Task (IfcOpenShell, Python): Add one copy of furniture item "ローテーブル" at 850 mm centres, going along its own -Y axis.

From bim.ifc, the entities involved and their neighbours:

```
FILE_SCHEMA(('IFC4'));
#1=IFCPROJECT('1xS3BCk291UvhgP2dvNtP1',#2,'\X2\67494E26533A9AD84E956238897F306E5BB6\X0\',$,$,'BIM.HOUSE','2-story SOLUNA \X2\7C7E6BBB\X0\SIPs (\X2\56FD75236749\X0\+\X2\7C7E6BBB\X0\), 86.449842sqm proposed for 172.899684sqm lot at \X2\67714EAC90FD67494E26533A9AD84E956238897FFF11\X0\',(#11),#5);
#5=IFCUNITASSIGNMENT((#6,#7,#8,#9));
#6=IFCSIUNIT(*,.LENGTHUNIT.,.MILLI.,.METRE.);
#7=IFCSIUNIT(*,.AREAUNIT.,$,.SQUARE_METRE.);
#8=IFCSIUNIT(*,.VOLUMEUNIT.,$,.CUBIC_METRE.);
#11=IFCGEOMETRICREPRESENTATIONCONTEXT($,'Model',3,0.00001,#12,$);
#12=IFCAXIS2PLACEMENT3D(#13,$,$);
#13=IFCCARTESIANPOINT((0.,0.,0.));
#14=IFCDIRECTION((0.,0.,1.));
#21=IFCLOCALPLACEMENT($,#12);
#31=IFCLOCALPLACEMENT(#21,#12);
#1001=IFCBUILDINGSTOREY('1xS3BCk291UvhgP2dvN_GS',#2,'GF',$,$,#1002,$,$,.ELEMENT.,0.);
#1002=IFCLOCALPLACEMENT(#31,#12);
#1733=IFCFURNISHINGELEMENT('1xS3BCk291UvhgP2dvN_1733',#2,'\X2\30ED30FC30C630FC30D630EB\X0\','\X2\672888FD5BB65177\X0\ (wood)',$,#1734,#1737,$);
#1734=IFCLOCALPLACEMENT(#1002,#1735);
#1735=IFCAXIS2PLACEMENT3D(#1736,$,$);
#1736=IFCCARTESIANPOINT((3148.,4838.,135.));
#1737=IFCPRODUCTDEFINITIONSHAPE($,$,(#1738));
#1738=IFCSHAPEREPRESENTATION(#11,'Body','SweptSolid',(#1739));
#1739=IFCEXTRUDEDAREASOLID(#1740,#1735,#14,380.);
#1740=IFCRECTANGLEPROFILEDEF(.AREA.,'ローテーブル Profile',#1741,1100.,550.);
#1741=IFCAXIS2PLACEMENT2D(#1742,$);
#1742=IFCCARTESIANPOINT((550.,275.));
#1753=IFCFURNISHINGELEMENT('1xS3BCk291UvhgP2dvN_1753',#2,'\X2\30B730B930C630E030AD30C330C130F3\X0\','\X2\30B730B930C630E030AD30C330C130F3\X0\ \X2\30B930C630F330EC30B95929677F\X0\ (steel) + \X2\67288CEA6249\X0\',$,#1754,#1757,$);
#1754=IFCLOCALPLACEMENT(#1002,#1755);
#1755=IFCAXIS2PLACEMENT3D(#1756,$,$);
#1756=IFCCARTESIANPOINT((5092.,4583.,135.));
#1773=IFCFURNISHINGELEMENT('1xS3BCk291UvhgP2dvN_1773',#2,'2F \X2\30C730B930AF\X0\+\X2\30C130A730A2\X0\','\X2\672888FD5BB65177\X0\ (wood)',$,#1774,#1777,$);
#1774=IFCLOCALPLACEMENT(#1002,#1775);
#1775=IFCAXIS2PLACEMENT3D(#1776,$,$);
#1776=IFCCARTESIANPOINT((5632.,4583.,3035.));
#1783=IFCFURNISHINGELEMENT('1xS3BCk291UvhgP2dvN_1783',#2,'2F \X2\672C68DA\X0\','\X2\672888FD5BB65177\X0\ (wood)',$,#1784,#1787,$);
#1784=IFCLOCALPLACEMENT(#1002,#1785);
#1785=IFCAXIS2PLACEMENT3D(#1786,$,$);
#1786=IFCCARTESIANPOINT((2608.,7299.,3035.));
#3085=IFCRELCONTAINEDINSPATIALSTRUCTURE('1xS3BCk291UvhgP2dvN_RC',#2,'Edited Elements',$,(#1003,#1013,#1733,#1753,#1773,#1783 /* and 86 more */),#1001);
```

```python
import ifcopenshell
import ifcopenshell.api.geometry
import ifcopenshell.api.root
import ifcopenshell.util.element
import ifcopenshell.util.placement
import ifcopenshell.util.unit

model = ifcopenshell.open("bim.ifc")
unit_scale = ifcopenshell.util.unit.calculate_unit_scale(model)


def reuse_history(source, copy):
    """copy_class also copies each property set's owner history, people and application; keep the originals."""
    for rel in copy.IsDefinedBy:
        if rel.is_a("IfcRelDefinesByProperties") and (history := rel.RelatingPropertyDefinition.OwnerHistory):
            rel.RelatingPropertyDefinition.OwnerHistory = source.OwnerHistory
            ifcopenshell.util.element.remove_deep2(model, history)


source = model.by_id(1733)
base = ifcopenshell.util.placement.get_local_placement(source.ObjectPlacement)
step = -base[:3, 1] * 0.85 / unit_scale

for i in range(1, 2):
    copy = ifcopenshell.api.root.copy_class(model, product=source)
    copy.Representation = ifcopenshell.util.element.copy_deep(
        model, source.Representation, exclude=["IfcGeometricRepresentationContext", "IfcRepresentationMap"]
    )
    reuse_history(source, copy)
    matrix = base.copy()
    matrix[:3, 3] += i * step
    print("added at", matrix[:3, 3].round(3) + 0.0)
    ifcopenshell.api.geometry.edit_object_placement(model, product=copy, matrix=matrix, is_si=False)

model.write("bim_v2.ifc")
```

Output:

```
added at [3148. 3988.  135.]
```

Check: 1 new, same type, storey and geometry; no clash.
